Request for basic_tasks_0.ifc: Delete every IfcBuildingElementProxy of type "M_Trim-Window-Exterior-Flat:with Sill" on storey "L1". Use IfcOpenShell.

First a look at what the model holds.

```python
import ifcopenshell
import ifcopenshell.util.element

model = ifcopenshell.open("basic_tasks_0.ifc")
print(model.schema)
storey = next(s for s in model.by_type("IfcBuildingStorey") if s.Name == "L1")
proxies = [e for e in ifcopenshell.util.element.get_decomposition(storey) if e.is_a("IfcBuildingElementProxy")]
seen = {}
for e in proxies:
    element_type = ifcopenshell.util.element.get_type(e)
    name = element_type.Name if element_type not in (None, e) else None
    seen[name] = seen.get(name, 0) + 1
for name, count in sorted(seen.items(), key=str):
    print(count, "x", name)
```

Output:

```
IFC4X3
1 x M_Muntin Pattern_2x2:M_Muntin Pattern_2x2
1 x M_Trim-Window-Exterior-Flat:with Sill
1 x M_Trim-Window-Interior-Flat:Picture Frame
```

```python
import ifcopenshell
import ifcopenshell.api.root
import ifcopenshell.util.element

model = ifcopenshell.open("basic_tasks_0.ifc")

storey = next(s for s in model.by_type("IfcBuildingStorey") if s.Name == "L1")
proxies = [e for e in ifcopenshell.util.element.get_decomposition(storey) if e.is_a("IfcBuildingElementProxy")]
targets = [e for e in proxies if (t := ifcopenshell.util.element.get_type(e)) not in (None, e) and t.Name == "M_Trim-Window-Exterior-Flat:with Sill"]

for e in targets:
    ifcopenshell.api.root.remove_product(model, product=e)
print(len(targets), "removed")

model.write("basic_tasks_0_edited.ifc")
```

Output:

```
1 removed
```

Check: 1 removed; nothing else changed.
